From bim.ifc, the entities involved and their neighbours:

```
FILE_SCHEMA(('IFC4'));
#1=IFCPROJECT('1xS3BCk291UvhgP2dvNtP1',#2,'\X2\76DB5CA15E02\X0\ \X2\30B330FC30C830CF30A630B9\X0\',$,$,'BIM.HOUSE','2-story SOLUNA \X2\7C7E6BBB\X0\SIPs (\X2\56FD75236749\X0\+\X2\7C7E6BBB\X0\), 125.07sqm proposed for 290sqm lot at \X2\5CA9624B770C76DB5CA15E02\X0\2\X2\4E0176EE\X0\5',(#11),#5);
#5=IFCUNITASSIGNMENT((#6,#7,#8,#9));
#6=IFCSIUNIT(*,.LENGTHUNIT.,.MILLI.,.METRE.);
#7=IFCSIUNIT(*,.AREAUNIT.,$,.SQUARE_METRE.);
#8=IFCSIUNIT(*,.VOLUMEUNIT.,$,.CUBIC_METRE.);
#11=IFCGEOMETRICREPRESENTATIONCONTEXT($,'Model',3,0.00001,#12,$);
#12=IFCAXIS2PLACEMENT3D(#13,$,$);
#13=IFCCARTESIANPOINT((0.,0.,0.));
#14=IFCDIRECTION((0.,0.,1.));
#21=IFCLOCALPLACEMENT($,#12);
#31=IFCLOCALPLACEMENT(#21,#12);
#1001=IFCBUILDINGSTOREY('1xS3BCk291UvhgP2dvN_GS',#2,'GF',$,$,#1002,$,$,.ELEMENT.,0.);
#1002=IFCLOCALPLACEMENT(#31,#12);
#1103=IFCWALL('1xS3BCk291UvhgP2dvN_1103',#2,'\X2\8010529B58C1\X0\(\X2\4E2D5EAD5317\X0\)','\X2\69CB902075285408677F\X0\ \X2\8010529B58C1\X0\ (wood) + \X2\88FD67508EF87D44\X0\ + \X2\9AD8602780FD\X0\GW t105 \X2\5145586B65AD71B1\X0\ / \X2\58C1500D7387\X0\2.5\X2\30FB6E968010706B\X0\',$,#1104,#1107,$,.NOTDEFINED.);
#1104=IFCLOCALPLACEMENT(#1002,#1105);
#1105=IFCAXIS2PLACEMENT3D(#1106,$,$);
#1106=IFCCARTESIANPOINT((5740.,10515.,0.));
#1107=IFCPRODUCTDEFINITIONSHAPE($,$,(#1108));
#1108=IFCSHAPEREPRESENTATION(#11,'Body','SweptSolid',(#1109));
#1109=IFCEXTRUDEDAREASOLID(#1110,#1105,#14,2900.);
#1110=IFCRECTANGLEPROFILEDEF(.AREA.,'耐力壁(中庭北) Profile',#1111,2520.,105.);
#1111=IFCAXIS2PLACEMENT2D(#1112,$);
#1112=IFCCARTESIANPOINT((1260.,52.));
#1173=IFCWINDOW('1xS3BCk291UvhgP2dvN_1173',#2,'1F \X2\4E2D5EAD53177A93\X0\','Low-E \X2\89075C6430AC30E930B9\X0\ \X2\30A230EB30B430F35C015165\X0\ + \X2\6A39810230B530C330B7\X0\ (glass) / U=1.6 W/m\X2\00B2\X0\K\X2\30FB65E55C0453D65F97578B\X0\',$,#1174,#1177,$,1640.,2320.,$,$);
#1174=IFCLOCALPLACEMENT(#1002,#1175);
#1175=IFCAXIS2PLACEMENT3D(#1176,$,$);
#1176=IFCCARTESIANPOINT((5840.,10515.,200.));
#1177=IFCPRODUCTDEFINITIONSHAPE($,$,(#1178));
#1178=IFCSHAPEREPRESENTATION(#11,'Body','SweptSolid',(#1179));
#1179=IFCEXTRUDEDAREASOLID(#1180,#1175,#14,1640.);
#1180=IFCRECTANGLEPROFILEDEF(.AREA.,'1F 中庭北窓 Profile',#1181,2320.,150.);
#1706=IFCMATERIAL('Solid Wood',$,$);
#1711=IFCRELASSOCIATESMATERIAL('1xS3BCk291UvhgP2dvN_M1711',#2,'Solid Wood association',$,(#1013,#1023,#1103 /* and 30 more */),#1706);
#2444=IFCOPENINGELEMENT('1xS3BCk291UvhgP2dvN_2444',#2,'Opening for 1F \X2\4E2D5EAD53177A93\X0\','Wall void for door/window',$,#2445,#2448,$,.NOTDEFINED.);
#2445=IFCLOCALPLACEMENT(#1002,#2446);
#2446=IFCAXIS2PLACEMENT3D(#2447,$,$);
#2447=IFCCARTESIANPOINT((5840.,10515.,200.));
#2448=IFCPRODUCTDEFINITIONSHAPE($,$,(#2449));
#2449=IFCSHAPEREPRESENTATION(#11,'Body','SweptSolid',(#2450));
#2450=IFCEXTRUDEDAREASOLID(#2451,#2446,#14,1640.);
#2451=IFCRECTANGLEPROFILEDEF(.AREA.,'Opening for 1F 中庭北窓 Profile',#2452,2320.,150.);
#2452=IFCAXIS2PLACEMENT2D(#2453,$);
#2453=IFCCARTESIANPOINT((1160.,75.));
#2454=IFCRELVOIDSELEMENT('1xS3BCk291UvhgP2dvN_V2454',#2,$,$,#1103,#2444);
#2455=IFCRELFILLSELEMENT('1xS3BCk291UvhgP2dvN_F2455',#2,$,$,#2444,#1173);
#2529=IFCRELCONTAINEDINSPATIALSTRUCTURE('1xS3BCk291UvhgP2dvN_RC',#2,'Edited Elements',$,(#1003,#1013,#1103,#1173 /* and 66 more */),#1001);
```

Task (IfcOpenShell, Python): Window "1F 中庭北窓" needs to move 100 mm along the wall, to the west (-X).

```python
import ifcopenshell
import ifcopenshell.api.geometry
import ifcopenshell.util.placement
import ifcopenshell.util.unit

model = ifcopenshell.open("bim.ifc")
unit_scale = ifcopenshell.util.unit.calculate_unit_scale(model)

window = model.by_guid("1xS3BCk291UvhgP2dvN_1173")
opening = window.FillsVoids[0].RelatingOpeningElement
wall = opening.VoidsElements[0].RelatingBuildingElement

wall_matrix = ifcopenshell.util.placement.get_local_placement(wall.ObjectPlacement)
shift = wall_matrix[:3, 0] * -0.1 / unit_scale
before = ifcopenshell.util.placement.get_local_placement(window.ObjectPlacement)[:3, 3].copy()

# The window is not placed relative to its opening, so move both.
for product in (opening, window):
    matrix = ifcopenshell.util.placement.get_local_placement(product.ObjectPlacement)
    matrix[:3, 3] += shift
    ifcopenshell.api.geometry.edit_object_placement(model, product=product, matrix=matrix, is_si=False)

after = ifcopenshell.util.placement.get_local_placement(window.ObjectPlacement)[:3, 3]
print("window moved by", (after - before).round(3) + 0.0)

model.write("bim_v2.ifc")
```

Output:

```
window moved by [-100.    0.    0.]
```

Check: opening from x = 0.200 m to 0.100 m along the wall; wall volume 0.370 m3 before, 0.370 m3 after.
